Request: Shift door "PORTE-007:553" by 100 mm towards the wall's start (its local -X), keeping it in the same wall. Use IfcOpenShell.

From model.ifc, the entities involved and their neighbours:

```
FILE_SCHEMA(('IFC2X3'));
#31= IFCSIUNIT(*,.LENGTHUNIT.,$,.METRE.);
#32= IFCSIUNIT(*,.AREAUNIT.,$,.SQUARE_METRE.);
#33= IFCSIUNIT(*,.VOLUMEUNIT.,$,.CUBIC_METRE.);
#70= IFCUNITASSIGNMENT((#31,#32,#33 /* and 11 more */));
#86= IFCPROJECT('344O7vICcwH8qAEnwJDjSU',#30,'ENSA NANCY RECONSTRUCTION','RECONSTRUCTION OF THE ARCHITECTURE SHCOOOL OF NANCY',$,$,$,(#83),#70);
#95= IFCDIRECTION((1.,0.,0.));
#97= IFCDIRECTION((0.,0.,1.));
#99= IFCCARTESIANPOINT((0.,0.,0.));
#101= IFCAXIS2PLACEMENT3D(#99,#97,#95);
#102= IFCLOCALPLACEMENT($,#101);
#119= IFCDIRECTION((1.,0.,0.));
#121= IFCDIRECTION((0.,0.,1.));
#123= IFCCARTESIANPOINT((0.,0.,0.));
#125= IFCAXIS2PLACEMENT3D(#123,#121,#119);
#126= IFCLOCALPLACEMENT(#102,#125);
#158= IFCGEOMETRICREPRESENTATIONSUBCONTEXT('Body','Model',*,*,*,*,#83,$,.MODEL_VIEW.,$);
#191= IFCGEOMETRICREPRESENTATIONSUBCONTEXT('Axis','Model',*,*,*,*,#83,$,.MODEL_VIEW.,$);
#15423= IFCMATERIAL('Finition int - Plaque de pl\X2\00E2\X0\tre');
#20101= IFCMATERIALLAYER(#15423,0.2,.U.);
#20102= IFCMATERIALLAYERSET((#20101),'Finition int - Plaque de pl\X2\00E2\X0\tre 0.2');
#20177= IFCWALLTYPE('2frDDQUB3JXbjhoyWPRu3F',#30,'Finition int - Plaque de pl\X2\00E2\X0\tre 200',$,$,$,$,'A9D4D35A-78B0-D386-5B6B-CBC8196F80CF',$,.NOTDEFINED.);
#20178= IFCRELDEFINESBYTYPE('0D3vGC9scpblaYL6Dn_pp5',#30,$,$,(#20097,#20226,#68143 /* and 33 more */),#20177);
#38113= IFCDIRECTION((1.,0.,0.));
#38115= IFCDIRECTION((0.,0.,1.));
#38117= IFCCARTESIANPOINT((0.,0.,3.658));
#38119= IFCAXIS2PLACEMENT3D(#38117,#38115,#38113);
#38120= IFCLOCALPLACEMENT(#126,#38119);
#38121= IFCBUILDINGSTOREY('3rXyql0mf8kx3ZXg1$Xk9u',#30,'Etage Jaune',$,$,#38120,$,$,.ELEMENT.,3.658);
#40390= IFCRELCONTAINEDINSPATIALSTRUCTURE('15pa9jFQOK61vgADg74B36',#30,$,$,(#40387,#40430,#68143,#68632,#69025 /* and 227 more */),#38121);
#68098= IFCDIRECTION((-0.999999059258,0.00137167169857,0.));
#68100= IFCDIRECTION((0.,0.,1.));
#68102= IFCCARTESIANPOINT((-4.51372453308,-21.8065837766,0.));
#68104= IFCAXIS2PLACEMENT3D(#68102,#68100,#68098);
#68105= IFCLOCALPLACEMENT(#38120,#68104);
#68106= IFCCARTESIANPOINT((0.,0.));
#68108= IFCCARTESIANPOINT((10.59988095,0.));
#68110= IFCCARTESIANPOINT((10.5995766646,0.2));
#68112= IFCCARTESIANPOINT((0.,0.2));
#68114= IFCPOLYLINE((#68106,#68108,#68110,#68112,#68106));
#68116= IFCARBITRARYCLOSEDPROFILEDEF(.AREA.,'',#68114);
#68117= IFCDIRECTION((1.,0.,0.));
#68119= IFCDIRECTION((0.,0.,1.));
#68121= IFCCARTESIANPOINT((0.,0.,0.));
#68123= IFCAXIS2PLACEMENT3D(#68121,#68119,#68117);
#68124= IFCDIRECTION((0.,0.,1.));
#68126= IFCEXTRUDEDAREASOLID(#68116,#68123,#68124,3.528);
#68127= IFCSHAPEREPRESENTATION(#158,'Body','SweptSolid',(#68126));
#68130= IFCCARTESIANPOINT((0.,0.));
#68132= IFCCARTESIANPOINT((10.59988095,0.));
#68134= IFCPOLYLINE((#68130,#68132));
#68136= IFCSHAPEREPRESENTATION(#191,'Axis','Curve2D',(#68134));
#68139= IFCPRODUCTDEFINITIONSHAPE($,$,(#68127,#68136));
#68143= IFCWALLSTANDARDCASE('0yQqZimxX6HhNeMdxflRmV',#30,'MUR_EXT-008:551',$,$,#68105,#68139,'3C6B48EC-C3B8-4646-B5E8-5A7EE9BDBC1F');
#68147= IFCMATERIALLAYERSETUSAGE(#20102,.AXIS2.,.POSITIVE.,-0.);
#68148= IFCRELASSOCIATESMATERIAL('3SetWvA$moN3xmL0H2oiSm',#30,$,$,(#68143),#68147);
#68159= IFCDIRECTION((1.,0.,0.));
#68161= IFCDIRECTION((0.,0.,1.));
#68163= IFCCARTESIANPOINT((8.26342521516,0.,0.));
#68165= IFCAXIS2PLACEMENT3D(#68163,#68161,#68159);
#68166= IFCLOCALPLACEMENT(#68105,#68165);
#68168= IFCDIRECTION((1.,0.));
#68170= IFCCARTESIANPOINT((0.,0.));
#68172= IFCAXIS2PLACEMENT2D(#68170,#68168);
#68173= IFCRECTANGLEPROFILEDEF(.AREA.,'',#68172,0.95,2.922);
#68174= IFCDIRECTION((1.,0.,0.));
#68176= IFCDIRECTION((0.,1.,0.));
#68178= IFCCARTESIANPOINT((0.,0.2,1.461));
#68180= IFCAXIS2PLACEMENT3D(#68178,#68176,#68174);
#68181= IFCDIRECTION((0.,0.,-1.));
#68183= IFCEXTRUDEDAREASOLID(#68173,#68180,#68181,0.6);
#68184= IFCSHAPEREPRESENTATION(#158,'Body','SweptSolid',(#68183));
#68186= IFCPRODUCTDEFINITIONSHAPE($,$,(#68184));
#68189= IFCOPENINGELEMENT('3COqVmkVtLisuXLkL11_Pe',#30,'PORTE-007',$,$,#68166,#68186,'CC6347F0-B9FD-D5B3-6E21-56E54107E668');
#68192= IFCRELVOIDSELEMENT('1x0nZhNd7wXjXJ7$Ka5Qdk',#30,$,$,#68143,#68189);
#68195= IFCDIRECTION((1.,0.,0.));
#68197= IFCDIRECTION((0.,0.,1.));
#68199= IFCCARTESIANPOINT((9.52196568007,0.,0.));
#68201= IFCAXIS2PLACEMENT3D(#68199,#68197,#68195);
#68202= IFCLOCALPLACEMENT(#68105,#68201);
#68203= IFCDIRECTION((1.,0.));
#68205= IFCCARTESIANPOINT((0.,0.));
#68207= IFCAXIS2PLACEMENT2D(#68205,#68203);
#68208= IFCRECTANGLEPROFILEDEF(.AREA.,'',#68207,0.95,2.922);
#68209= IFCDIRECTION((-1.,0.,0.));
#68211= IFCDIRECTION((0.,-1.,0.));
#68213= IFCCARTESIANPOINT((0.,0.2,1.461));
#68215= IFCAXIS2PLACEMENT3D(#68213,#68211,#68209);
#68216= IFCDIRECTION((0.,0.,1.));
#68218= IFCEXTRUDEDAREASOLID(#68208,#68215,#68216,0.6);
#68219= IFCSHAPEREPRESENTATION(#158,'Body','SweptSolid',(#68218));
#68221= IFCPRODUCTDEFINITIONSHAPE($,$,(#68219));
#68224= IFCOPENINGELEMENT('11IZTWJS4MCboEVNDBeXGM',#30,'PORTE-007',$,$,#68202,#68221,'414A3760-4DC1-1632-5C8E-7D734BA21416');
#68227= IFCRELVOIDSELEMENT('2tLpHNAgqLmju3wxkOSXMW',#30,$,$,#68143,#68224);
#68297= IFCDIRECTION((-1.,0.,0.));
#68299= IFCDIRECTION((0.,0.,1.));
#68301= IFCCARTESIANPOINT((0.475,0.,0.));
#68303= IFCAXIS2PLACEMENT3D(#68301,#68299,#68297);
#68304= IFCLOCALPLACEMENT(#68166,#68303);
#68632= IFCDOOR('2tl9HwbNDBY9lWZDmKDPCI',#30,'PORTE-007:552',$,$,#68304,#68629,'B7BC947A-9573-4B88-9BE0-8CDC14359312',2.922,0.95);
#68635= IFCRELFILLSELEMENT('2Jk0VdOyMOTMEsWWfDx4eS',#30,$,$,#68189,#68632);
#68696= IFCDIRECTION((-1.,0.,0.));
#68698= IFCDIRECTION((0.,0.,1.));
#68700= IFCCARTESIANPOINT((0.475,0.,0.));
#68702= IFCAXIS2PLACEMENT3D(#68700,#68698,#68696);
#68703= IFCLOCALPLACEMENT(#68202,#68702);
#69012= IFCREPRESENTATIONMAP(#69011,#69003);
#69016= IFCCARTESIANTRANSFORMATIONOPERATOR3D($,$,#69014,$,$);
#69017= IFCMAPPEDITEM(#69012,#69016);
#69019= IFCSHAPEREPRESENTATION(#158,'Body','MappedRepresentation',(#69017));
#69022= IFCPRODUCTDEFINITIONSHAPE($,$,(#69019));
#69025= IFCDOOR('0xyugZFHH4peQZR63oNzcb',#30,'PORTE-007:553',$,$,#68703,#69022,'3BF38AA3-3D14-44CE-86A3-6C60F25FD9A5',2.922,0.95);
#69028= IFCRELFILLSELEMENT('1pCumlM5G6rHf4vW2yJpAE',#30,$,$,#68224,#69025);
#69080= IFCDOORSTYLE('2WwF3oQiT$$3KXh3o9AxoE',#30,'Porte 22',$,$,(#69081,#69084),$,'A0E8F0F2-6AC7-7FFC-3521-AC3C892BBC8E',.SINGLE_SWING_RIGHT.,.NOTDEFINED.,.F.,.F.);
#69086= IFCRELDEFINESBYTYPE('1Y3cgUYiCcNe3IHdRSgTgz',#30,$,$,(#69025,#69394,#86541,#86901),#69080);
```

```python
import ifcopenshell
import ifcopenshell.api.geometry
import ifcopenshell.util.placement

model = ifcopenshell.open("model.ifc")

door = model.by_guid("0xyugZFHH4peQZR63oNzcb")
opening = door.FillsVoids[0].RelatingOpeningElement
wall = opening.VoidsElements[0].RelatingBuildingElement

wall_matrix = ifcopenshell.util.placement.get_local_placement(wall.ObjectPlacement)
shift = wall_matrix[:3, 0] * -0.1
before = ifcopenshell.util.placement.get_local_placement(door.ObjectPlacement)[:3, 3].copy()

# The door is placed relative to its opening, so it follows when the opening moves.
matrix = ifcopenshell.util.placement.get_local_placement(opening.ObjectPlacement)
matrix[:3, 3] += shift
ifcopenshell.api.geometry.edit_object_placement(
    model, product=opening, matrix=matrix, is_si=False, should_transform_children=True
)

after = ifcopenshell.util.placement.get_local_placement(door.ObjectPlacement)[:3, 3]
print("door moved by", (after - before).round(3) + 0.0)

model.write("model_v2.ifc")
```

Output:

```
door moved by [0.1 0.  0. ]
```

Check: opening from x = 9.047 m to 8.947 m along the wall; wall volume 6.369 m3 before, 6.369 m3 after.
